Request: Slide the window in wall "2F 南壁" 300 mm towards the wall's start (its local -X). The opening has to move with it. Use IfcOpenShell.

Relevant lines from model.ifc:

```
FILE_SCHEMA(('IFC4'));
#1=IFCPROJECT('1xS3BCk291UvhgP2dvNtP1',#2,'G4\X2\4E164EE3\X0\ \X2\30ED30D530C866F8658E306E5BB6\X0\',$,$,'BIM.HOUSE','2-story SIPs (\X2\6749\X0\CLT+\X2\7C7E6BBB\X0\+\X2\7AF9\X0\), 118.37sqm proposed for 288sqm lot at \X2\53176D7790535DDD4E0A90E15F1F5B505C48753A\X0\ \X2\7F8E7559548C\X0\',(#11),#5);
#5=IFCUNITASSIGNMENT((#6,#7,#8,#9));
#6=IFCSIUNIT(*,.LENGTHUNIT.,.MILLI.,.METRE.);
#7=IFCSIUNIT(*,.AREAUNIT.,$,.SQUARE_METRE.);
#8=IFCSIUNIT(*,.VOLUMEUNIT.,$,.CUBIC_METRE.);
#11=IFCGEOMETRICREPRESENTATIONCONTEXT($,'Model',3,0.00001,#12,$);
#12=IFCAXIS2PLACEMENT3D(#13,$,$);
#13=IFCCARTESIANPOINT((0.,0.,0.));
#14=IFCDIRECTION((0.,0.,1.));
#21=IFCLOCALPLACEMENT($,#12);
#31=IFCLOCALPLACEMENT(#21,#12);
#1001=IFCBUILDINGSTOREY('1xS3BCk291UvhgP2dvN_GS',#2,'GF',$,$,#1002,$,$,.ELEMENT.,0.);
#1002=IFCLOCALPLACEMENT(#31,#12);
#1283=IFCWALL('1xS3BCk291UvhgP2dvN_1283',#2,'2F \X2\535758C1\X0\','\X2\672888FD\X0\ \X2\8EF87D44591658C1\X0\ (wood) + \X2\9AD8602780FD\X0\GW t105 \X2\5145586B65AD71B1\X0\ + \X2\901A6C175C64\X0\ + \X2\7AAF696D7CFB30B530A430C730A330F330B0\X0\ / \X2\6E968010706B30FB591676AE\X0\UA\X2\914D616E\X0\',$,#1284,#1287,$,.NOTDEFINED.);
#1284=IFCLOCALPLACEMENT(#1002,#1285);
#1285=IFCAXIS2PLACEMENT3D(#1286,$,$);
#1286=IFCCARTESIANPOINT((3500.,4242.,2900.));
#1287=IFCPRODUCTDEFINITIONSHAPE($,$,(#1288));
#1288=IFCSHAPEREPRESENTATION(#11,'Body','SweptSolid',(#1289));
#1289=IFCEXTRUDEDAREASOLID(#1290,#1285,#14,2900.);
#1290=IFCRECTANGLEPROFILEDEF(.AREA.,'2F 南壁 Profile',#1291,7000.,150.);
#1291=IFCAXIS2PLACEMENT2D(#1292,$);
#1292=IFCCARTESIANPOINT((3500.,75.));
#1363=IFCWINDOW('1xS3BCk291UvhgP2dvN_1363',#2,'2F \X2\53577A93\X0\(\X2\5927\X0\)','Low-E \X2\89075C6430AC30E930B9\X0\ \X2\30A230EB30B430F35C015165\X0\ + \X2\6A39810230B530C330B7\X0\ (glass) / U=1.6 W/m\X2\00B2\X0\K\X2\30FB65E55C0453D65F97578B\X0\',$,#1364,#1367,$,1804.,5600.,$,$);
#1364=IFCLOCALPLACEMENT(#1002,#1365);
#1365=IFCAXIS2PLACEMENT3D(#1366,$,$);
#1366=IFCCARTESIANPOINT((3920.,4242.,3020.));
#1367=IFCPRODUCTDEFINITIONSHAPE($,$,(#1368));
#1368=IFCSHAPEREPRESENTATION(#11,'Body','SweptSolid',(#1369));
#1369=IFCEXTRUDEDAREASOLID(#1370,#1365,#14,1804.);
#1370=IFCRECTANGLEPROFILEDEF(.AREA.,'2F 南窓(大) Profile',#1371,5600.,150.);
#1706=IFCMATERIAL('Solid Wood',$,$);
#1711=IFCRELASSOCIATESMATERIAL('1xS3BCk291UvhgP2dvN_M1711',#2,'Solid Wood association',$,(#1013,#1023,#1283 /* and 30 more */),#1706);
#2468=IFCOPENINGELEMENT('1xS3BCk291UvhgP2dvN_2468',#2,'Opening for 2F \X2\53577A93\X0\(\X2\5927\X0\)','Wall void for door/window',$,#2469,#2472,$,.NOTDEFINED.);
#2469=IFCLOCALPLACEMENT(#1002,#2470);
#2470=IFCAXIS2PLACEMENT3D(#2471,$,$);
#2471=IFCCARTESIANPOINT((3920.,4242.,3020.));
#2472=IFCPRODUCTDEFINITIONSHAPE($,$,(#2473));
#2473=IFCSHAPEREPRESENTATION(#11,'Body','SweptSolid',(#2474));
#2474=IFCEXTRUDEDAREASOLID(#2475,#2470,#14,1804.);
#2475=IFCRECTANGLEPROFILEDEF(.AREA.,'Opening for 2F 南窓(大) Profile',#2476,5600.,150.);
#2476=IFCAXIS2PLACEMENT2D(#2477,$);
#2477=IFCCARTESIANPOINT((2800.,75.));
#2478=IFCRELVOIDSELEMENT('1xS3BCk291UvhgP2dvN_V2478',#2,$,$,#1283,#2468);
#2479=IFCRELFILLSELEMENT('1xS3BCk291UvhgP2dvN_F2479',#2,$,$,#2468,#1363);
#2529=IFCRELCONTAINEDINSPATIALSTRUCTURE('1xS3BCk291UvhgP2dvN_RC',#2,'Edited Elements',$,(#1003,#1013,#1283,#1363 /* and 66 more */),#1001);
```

```python
import ifcopenshell
import ifcopenshell.api.geometry
import ifcopenshell.util.placement

model = ifcopenshell.open("model.ifc")

window = model.by_guid("1xS3BCk291UvhgP2dvN_1363")
opening = window.FillsVoids[0].RelatingOpeningElement
wall = opening.VoidsElements[0].RelatingBuildingElement

wall_matrix = ifcopenshell.util.placement.get_local_placement(wall.ObjectPlacement)
shift = wall_matrix[:3, 0] * -300.0
before = ifcopenshell.util.placement.get_local_placement(window.ObjectPlacement)[:3, 3].copy()

# The window is not placed relative to its opening, so move both.
for product in (opening, window):
    matrix = ifcopenshell.util.placement.get_local_placement(product.ObjectPlacement)
    matrix[:3, 3] += shift
    ifcopenshell.api.geometry.edit_object_placement(model, product=product, matrix=matrix, is_si=False)

after = ifcopenshell.util.placement.get_local_placement(window.ObjectPlacement)[:3, 3]
print("window moved by", (after - before).round(3) + 0.0)

model.write("model-out.ifc")
```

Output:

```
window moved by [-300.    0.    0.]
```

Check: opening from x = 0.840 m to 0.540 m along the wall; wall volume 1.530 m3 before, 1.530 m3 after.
